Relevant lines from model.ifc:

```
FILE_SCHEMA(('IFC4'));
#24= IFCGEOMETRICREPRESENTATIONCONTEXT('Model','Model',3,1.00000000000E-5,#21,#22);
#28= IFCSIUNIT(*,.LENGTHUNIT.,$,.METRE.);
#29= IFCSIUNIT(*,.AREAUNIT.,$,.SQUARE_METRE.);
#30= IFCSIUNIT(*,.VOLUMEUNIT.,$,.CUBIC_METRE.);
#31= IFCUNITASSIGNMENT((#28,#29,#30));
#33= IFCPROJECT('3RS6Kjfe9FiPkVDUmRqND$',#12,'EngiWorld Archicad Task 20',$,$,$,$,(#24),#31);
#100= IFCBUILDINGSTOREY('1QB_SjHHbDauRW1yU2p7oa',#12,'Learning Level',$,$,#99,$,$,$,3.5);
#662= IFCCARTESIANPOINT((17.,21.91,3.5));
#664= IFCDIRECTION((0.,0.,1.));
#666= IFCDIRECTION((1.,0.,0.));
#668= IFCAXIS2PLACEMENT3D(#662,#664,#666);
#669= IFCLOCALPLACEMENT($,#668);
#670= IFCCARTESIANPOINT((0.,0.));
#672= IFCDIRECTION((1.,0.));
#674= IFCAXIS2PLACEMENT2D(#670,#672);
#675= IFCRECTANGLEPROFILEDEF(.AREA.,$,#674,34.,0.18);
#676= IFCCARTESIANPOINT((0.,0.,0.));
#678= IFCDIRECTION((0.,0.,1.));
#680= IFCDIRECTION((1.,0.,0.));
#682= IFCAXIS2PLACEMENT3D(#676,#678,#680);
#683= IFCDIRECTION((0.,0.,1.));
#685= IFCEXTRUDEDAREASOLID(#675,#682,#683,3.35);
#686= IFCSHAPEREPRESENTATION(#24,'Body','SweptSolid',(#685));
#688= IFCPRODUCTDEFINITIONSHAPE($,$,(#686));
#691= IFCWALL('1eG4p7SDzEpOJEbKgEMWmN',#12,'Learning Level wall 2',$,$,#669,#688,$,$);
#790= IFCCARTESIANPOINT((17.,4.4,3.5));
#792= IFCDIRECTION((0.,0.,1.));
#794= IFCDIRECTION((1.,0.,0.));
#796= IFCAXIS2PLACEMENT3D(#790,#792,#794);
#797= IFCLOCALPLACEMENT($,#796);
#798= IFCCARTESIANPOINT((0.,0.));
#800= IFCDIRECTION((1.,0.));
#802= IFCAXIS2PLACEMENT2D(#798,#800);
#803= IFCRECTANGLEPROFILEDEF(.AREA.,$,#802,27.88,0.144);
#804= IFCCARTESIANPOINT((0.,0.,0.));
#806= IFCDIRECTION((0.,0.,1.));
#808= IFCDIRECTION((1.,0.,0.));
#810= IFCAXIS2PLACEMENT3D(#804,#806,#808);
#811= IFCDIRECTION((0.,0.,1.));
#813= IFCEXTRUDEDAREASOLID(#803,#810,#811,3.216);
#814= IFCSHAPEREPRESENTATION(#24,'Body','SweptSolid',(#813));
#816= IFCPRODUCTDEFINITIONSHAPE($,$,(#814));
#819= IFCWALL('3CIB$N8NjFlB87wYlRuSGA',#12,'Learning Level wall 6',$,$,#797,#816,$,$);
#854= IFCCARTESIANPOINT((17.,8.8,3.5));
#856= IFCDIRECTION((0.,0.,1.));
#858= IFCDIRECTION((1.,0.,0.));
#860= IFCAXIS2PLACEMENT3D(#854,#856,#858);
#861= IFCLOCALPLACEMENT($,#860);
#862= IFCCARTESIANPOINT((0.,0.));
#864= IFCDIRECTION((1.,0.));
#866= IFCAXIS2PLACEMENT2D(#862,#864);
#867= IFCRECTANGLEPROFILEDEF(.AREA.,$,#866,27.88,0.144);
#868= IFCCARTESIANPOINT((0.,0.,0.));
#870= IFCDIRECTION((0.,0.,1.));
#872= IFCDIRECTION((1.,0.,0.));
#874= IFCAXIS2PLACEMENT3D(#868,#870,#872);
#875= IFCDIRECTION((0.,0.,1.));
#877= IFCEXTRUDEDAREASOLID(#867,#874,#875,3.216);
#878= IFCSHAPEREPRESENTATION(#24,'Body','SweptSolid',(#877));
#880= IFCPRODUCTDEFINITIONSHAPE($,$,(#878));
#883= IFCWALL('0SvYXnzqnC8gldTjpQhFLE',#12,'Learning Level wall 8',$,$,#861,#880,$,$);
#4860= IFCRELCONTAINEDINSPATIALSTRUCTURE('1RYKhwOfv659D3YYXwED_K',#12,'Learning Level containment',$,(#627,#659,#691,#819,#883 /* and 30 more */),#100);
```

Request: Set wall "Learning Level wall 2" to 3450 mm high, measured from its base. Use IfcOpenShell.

```python
import ifcopenshell
import ifcopenshell.geom
import ifcopenshell.util.shape
import ifcopenshell.util.unit

model = ifcopenshell.open("model.ifc")
unit_scale = ifcopenshell.util.unit.calculate_unit_scale(model)
settings = ifcopenshell.geom.settings()


def volume(element):
    """Net volume in cubic metres, openings subtracted."""
    shape = ifcopenshell.geom.create_shape(settings, element)
    return ifcopenshell.util.shape.get_volume(shape.geometry)


wall = model.by_guid("1eG4p7SDzEpOJEbKgEMWmN")
before = volume(wall)

body = next(r for r in wall.Representation.Representations if r.RepresentationIdentifier == "Body")
solid = body.Items[0]
old_height = solid.Depth
solid.Depth = 3.45 / unit_scale
after = volume(wall)

print(f"height {old_height:g} -> {solid.Depth:g}, volume {before:.3f} -> {after:.3f} m3")

model.write("model-out.ifc")
```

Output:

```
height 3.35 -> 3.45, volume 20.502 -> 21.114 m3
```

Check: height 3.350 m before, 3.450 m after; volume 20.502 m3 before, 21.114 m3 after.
